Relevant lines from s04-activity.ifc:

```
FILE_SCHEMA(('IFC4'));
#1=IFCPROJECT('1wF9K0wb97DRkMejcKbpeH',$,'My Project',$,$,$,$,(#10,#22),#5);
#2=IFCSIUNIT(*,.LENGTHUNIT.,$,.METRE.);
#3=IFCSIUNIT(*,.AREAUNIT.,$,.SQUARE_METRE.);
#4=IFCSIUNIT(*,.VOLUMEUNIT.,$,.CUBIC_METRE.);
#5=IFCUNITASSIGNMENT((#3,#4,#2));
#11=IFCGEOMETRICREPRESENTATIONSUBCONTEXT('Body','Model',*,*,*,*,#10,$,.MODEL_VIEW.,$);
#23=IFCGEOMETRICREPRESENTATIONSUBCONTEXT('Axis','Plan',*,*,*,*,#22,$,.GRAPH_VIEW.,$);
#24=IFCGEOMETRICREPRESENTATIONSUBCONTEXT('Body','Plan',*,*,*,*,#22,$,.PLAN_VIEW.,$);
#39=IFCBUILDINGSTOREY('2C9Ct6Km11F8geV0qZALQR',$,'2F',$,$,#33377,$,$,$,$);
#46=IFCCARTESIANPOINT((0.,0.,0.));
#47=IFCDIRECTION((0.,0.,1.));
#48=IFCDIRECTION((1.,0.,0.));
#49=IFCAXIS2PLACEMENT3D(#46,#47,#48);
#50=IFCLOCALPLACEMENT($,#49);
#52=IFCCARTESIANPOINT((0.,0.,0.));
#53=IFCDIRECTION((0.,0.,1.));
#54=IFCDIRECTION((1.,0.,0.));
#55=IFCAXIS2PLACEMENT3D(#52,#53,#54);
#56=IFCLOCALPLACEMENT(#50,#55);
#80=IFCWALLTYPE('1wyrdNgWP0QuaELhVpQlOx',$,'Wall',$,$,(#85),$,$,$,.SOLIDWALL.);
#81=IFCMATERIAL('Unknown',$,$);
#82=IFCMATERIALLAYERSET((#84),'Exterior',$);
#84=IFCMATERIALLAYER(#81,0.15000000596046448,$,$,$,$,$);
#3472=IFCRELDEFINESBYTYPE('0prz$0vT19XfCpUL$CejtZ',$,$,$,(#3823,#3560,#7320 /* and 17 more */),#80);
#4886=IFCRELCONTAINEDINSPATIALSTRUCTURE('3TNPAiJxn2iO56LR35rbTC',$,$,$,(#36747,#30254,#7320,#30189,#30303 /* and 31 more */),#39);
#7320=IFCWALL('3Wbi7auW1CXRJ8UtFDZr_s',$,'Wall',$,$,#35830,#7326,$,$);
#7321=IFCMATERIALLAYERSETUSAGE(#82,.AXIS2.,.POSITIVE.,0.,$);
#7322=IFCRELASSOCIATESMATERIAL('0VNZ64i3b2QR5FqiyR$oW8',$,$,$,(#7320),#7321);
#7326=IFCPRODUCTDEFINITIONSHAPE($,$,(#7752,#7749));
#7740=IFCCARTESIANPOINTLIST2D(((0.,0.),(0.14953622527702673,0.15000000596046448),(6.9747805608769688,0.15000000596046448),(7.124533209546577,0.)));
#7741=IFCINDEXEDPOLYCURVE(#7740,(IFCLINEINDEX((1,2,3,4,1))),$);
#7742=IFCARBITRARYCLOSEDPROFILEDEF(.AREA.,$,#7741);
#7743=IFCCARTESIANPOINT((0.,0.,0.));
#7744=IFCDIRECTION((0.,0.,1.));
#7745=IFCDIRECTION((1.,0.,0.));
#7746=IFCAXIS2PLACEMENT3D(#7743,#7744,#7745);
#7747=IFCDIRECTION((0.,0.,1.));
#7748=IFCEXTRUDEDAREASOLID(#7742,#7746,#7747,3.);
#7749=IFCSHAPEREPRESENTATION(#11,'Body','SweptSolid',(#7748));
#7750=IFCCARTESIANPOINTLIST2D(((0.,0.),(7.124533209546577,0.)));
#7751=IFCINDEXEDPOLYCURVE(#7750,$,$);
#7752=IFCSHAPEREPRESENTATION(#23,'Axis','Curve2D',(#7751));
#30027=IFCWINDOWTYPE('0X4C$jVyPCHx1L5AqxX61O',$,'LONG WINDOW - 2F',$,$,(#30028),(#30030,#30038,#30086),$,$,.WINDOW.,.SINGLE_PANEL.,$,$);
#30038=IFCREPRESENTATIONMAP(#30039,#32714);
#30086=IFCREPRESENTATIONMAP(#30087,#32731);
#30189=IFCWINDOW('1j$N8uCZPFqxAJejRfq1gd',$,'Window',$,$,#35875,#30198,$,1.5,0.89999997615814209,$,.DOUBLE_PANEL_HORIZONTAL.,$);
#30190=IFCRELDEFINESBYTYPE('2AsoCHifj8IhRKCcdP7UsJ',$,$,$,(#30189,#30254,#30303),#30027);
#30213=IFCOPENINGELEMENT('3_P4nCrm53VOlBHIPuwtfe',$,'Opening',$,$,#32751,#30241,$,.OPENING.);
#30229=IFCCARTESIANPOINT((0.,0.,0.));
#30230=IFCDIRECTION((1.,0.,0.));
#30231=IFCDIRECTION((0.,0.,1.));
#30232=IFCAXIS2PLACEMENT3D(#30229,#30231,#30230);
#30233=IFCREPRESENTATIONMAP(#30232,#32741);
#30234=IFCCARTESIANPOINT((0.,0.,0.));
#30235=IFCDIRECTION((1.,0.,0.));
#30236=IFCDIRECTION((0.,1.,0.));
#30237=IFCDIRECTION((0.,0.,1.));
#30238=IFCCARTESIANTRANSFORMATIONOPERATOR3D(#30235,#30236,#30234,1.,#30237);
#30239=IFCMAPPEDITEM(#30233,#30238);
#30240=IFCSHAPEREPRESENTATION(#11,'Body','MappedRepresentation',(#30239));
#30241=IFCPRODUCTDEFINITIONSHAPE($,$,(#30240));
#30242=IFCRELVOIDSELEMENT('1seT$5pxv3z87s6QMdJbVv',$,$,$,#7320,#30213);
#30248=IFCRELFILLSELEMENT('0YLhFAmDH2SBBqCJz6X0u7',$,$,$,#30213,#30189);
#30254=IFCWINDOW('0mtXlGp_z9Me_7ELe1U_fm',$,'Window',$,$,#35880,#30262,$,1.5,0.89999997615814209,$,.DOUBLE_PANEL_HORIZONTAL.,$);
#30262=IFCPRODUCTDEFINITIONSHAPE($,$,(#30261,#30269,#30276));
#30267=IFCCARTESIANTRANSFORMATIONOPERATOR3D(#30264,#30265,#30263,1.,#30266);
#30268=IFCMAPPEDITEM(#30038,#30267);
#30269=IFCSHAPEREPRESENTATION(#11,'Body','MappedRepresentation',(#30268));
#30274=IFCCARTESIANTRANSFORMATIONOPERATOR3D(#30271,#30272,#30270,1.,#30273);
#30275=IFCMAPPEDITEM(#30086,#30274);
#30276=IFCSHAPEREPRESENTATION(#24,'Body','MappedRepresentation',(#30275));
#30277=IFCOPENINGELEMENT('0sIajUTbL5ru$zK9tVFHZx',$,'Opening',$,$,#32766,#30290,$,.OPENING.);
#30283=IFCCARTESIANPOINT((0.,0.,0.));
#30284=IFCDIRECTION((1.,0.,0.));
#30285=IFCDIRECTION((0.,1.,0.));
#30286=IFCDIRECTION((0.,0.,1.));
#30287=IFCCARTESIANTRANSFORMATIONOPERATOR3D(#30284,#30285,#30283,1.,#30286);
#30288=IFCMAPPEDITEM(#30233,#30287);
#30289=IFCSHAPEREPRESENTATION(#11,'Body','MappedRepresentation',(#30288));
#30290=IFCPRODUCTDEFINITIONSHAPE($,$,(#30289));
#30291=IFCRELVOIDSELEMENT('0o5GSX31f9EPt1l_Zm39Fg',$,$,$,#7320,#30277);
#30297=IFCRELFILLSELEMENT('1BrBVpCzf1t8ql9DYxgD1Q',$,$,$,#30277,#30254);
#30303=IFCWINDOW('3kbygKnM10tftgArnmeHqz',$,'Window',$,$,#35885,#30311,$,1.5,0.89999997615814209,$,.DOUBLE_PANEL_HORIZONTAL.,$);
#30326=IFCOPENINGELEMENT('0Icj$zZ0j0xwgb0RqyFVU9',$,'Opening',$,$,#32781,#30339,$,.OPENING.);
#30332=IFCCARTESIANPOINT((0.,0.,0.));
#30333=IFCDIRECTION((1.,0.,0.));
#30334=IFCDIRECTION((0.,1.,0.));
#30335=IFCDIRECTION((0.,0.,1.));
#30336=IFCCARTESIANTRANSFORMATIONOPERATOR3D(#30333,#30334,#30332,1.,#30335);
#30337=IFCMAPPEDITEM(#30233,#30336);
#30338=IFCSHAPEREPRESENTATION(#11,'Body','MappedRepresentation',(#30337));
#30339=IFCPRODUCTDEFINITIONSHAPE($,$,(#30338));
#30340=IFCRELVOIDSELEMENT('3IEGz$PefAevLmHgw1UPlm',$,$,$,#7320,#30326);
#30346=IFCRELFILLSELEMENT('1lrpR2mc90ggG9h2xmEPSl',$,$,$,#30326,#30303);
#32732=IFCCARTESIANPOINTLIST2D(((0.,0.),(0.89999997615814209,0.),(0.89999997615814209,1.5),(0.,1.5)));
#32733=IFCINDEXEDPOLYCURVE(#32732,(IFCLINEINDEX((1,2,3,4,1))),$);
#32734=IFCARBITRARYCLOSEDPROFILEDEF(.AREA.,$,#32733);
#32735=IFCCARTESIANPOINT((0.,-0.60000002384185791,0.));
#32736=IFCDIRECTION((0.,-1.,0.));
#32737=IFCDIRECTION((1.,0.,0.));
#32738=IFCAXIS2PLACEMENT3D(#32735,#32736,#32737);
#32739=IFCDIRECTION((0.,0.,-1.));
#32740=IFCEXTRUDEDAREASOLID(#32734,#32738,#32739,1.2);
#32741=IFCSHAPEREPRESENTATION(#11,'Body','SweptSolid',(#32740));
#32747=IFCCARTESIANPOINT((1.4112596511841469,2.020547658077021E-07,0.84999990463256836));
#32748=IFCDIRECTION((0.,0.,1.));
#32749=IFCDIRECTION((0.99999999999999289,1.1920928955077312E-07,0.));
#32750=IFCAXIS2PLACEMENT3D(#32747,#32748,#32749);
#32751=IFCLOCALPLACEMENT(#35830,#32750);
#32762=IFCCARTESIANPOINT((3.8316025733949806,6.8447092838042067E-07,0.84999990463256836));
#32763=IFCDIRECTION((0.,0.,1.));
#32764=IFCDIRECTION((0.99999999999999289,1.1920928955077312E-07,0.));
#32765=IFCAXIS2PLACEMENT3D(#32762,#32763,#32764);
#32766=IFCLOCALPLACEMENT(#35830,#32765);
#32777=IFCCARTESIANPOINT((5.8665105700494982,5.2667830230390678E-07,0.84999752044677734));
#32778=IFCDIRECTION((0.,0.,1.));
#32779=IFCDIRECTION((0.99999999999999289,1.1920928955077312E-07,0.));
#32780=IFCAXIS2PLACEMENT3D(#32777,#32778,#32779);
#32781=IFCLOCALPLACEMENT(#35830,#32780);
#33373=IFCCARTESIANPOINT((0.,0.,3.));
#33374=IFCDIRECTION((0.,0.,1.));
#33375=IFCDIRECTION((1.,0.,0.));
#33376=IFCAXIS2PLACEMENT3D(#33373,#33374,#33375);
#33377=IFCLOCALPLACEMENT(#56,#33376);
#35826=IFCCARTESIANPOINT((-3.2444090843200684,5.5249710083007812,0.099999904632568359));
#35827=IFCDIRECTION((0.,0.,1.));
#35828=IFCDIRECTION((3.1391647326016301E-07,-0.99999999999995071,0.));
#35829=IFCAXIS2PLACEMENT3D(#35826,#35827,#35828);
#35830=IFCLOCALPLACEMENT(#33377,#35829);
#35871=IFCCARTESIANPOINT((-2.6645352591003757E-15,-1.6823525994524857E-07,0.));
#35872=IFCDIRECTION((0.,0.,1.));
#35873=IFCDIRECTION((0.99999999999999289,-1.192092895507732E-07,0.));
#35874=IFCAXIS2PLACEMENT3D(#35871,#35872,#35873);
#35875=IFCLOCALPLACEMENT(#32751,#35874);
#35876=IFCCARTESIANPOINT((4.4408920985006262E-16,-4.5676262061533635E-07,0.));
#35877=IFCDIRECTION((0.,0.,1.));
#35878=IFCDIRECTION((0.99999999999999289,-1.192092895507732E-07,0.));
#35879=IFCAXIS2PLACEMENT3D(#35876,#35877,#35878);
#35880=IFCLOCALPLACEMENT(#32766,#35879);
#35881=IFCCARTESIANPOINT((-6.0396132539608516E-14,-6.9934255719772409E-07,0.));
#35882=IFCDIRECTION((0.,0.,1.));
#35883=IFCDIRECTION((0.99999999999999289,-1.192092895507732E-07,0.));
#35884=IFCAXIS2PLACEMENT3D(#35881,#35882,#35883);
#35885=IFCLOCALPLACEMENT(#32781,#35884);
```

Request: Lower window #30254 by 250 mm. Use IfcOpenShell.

```python
import numpy as np
import ifcopenshell
import ifcopenshell.api.geometry
import ifcopenshell.util.placement
import ifcopenshell.util.unit

model = ifcopenshell.open("s04-activity.ifc")
unit_scale = ifcopenshell.util.unit.calculate_unit_scale(model)

window = model.by_guid("0mtXlGp_z9Me_7ELe1U_fm")
opening = window.FillsVoids[0].RelatingOpeningElement
dz = -0.25

shift = np.array([0.0, 0.0, dz])
# The window is placed relative to its opening, so it follows when the opening moves.
matrix = ifcopenshell.util.placement.get_local_placement(opening.ObjectPlacement)
matrix[:3, 3] += shift
ifcopenshell.api.geometry.edit_object_placement(
    model, product=opening, matrix=matrix, is_si=False, should_transform_children=True
)

print(f"moved by {dz * unit_scale:+.3f} m")

model.write("s04-activity_updated.ifc")
```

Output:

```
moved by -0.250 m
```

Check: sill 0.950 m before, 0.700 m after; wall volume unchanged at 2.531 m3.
